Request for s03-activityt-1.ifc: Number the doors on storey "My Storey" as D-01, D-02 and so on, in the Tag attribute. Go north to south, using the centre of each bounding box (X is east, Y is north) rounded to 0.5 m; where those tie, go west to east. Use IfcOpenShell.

First a look at what the model holds.

```python
import ifcopenshell
import ifcopenshell.util.element
import ifcopenshell.util.placement

model = ifcopenshell.open("s03-activityt-1.ifc")
print(model.schema)
storey = next(s for s in model.by_type("IfcBuildingStorey") if s.Name == "My Storey")
doors = [e for e in ifcopenshell.util.element.get_decomposition(storey) if e.is_a("IfcDoor")]
for e in sorted(doors, key=lambda e: e.id()):
    origin = ifcopenshell.util.placement.get_local_placement(e.ObjectPlacement)[:3, 3]
    print(e.id(), e.Tag, e.Name, origin.round(2) + 0.0, sep=" | ")
```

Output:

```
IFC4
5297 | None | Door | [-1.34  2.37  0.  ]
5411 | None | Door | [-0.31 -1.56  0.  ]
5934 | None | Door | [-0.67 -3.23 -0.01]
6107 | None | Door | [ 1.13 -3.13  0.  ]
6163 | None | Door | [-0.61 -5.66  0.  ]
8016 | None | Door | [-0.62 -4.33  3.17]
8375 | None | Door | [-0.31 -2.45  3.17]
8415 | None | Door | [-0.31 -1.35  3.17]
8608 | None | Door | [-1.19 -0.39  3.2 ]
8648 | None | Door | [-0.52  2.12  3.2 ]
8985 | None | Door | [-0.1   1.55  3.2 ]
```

```python
import ifcopenshell
import ifcopenshell.geom
import ifcopenshell.util.element
import ifcopenshell.util.shape

model = ifcopenshell.open("s03-activityt-1.ifc")
settings = ifcopenshell.geom.settings()
settings.set("use-world-coords", True)


def centre(element):
    shape = ifcopenshell.geom.create_shape(settings, element)
    return ifcopenshell.util.shape.get_bbox_centroid(shape.geometry)


storey = next(s for s in model.by_type("IfcBuildingStorey") if s.Name == "My Storey")
doors = [e for e in ifcopenshell.util.element.get_decomposition(storey) if e.is_a("IfcDoor")]

# Insertion points can sit at a corner or the storey origin, so sort by the geometry (in metres).
centres = {e: centre(e) for e in doors}
doors.sort(key=lambda e: (-round(centres[e][1] / 0.5), centres[e][0]))

for i, e in enumerate(doors, start=1):
    number = f"D-{i:02d}"
    e.Tag = number
    print(e.id(), number)

model.write("s03-activityt-1_edited.ifc")
```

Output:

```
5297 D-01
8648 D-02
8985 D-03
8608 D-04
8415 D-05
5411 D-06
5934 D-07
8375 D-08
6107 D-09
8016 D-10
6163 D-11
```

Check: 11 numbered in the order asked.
